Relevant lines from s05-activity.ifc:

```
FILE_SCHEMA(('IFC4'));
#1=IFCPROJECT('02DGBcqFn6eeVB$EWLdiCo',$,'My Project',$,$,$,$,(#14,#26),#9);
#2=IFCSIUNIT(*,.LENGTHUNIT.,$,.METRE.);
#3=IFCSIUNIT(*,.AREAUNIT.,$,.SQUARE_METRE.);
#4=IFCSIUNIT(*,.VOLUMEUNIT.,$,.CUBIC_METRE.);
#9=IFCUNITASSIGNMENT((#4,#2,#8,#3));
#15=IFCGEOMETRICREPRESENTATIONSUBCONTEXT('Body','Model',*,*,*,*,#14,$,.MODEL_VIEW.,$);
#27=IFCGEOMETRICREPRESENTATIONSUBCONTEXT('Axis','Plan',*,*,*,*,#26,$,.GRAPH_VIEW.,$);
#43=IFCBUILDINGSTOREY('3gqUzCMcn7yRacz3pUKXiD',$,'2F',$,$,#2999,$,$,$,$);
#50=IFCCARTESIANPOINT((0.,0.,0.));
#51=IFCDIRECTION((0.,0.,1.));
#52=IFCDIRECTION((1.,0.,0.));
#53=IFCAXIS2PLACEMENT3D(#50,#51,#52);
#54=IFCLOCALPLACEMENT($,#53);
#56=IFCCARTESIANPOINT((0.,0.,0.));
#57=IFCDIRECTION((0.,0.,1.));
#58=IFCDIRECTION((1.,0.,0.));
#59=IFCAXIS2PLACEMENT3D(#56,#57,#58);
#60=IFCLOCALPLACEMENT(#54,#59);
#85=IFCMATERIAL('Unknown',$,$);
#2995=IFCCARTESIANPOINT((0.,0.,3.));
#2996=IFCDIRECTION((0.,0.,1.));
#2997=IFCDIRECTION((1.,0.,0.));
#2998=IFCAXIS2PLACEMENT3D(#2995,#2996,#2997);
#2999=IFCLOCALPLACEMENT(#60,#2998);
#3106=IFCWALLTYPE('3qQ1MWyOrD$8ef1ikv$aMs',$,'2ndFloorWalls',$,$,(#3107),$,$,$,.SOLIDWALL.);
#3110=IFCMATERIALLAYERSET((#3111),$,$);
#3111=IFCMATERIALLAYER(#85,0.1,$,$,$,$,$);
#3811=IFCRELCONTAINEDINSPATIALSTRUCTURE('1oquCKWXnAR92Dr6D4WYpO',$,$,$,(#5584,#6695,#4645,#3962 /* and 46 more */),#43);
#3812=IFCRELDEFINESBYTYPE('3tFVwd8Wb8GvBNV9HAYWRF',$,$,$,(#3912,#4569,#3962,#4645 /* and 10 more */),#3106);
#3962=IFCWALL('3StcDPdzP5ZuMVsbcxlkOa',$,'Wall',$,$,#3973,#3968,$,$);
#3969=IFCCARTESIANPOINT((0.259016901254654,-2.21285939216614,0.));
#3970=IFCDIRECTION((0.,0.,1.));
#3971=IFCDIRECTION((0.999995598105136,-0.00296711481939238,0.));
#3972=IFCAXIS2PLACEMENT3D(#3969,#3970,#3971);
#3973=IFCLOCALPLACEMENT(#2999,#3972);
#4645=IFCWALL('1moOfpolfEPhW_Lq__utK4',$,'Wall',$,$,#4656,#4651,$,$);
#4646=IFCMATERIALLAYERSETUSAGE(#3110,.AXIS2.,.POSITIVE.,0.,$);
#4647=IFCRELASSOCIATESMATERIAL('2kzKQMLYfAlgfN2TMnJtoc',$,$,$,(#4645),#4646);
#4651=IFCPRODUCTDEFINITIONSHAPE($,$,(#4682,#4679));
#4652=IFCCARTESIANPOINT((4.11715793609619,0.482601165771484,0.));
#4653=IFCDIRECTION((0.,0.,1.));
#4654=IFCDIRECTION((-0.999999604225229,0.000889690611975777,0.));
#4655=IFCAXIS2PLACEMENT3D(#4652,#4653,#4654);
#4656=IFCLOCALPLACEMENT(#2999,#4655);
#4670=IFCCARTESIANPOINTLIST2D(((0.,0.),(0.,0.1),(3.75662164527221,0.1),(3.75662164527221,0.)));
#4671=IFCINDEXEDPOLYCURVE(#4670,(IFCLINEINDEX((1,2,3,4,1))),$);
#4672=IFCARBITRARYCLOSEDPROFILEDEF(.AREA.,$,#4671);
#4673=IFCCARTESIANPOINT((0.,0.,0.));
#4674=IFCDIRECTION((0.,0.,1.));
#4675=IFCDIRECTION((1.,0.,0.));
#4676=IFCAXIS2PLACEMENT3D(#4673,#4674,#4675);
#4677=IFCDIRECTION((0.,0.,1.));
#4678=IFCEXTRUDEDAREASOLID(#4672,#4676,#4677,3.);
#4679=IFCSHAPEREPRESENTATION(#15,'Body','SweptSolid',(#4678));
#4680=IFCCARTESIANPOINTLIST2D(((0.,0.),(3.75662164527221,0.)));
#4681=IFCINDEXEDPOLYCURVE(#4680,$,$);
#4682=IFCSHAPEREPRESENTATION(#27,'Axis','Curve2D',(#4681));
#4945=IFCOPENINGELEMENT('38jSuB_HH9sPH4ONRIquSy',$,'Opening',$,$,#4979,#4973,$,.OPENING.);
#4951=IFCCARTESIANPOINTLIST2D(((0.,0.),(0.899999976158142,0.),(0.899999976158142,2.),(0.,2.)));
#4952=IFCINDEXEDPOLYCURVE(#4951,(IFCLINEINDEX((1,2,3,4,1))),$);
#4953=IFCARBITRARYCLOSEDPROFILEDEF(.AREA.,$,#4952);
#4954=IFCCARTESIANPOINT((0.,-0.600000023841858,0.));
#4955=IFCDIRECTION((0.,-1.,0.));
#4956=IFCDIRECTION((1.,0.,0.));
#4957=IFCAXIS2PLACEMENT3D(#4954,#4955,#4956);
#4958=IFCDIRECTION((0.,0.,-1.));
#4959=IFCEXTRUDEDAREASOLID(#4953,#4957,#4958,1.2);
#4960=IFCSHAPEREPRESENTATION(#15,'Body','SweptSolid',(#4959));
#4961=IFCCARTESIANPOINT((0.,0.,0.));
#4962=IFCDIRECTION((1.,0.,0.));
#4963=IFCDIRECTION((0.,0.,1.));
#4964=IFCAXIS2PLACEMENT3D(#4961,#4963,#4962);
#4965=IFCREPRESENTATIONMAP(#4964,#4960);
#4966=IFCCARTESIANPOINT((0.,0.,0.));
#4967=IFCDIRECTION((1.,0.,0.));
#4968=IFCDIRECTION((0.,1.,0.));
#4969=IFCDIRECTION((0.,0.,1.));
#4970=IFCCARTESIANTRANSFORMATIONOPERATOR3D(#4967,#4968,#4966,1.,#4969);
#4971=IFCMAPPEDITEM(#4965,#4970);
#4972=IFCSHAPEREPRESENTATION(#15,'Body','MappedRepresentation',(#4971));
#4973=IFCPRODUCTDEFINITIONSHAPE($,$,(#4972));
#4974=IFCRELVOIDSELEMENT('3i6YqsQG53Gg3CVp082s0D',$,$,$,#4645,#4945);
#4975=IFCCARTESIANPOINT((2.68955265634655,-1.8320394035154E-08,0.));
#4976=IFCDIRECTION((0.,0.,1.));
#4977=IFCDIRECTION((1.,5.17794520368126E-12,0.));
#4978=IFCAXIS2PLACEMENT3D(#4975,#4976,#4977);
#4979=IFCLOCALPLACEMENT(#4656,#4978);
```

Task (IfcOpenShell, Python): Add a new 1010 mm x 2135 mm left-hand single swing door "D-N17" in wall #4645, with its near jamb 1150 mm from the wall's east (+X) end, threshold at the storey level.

```python
import numpy as np
import ifcopenshell
import ifcopenshell.api.feature
import ifcopenshell.api.geometry
import ifcopenshell.api.root
import ifcopenshell.api.spatial
import ifcopenshell.geom
import ifcopenshell.util.element
import ifcopenshell.util.placement
import ifcopenshell.util.representation
import ifcopenshell.util.shape
import ifcopenshell.util.unit

model = ifcopenshell.open("s05-activity.ifc")
unit_scale = ifcopenshell.util.unit.calculate_unit_scale(model)
settings = ifcopenshell.geom.settings()


def volume(element):
    """Net volume in cubic metres, openings subtracted."""
    shape = ifcopenshell.geom.create_shape(settings, element)
    return ifcopenshell.util.shape.get_volume(shape.geometry)


wall = model.by_guid("1moOfpolfEPhW_Lq__utK4")
storey = ifcopenshell.util.element.get_container(wall, ifc_class="IfcBuildingStorey")
context = ifcopenshell.util.representation.get_context(model, "Model", "Body", "MODEL_VIEW")
before = volume(wall)

width, height, from_end, sill = 1.01, 2.135, 1.15, 0.0  # metres

# The wall runs along its own X axis, and the end named is its -X end.
wall_shape = ifcopenshell.geom.create_shape(settings, wall)
x, y, z = ifcopenshell.util.shape.get_vertices(wall_shape.geometry).T
start = x.min() + from_end
face, thickness = float(y.min()), float(y.max() - y.min())
wall_matrix = ifcopenshell.util.placement.get_local_placement(wall.ObjectPlacement)
level = ifcopenshell.util.placement.get_local_placement(storey.ObjectPlacement)[2, 3]


def in_wall(x, y):
    """Placement at x, y metres in the wall's axes, at sill height."""
    matrix = wall_matrix.copy()
    matrix[:, 3] = wall_matrix @ np.array([x / unit_scale, y / unit_scale, 0.0, 1.0])
    matrix[2, 3] = level + sill / unit_scale
    return matrix


# Opening: a box that overshoots both wall faces by 50 mm.
opening = ifcopenshell.api.root.create_entity(model, ifc_class="IfcOpeningElement", predefined_type="OPENING")
box = ifcopenshell.api.geometry.add_wall_representation(
    model, context=context, length=width, height=height, thickness=thickness + 0.1
)
ifcopenshell.api.geometry.assign_representation(model, product=opening, representation=box)
ifcopenshell.api.geometry.edit_object_placement(model, product=opening, matrix=in_wall(start, face - 0.05), is_si=False)
ifcopenshell.api.feature.add_feature(model, feature=opening, element=wall)

door = ifcopenshell.api.root.create_entity(model, ifc_class="IfcDoor", name="D-N17", predefined_type="DOOR")
door.OverallWidth, door.OverallHeight = width / unit_scale, height / unit_scale
door.OperationType = "SINGLE_SWING_LEFT"
body = ifcopenshell.api.geometry.add_door_representation(
    model,
    context=context,
    overall_width=door.OverallWidth,
    overall_height=door.OverallHeight,
    operation_type="SINGLE_SWING_LEFT",
    lining_properties={"LiningDepth": thickness / unit_scale, "ThresholdDepth": thickness / unit_scale},
)
ifcopenshell.api.geometry.assign_representation(model, product=door, representation=body)
ifcopenshell.api.spatial.assign_container(model, products=[door], relating_structure=storey)
ifcopenshell.api.feature.add_filling(model, opening=opening, element=door)

# The lining spans the wall, so the door starts at the wall face.
ifcopenshell.api.geometry.edit_object_placement(model, product=door, matrix=in_wall(start, face), is_si=False)

after = volume(wall)

print(f"wall volume {before:.3f} -> {after:.3f} m3")

model.write("s05-activity_v2.ifc")
```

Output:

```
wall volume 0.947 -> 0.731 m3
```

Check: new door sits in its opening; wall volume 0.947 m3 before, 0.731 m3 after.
